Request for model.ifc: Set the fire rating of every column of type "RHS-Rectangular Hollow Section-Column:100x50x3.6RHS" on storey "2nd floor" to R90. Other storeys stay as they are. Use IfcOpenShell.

First a look at what the model holds.

```python
import ifcopenshell
import ifcopenshell.util.element

model = ifcopenshell.open("model.ifc")
print(model.schema)
storey = next(s for s in model.by_type("IfcBuildingStorey") if s.Name == "2nd floor")
columns = [e for e in ifcopenshell.util.element.get_decomposition(storey) if e.is_a("IfcColumn")]
seen = {}
for e in columns:
    element_type = ifcopenshell.util.element.get_type(e)
    key = (element_type.Name if element_type != e and element_type else None, ifcopenshell.util.element.get_pset(e, "Pset_ColumnCommon", "FireRating"))
    seen[key] = seen.get(key, 0) + 1
for (name, value), count in sorted(seen.items(), key=str):
    print(count, "x", name, "|", value)
```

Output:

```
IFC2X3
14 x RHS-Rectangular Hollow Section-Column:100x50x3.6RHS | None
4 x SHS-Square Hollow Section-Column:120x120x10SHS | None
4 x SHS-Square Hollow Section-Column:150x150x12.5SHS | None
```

```python
import ifcopenshell
import ifcopenshell.api.pset
import ifcopenshell.util.element

model = ifcopenshell.open("model.ifc")

storey = next(s for s in model.by_type("IfcBuildingStorey") if s.Name == "2nd floor")
columns = [e for e in ifcopenshell.util.element.get_decomposition(storey) if e.is_a("IfcColumn")]

count = 0
for e in columns:
    element_type = ifcopenshell.util.element.get_type(e)
    if element_type in (None, e) or element_type.Name != "RHS-Rectangular Hollow Section-Column:100x50x3.6RHS":
        continue
    # add_pset returns the element's existing set when there is one.
    pset = ifcopenshell.api.pset.add_pset(model, product=e, name="Pset_ColumnCommon")
    ifcopenshell.api.pset.edit_pset(model, pset=pset, properties={"FireRating": "R90"})
    count += 1

print(count, "columns updated")

model.write("model_edited.ifc")
```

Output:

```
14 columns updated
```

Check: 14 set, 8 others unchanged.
